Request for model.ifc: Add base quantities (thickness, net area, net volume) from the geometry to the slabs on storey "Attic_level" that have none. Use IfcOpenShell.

First a look at what the model holds.

```python
import ifcopenshell
import ifcopenshell.util.element
import ifcopenshell.util.unit

model = ifcopenshell.open("model.ifc")
print(model.schema)
for unit_type in ("LENGTHUNIT", "AREAUNIT", "VOLUMEUNIT"):
    print(unit_type, ifcopenshell.util.unit.calculate_unit_scale(model, unit_type))
storey = next(s for s in model.by_type("IfcBuildingStorey") if s.Name == "Attic_level")
slabs = [e for e in ifcopenshell.util.element.get_decomposition(storey) if e.is_a("IfcSlab")]
for e in sorted(slabs, key=lambda e: e.id()):
    print(e.id(), e.is_a(), e.Name, list(ifcopenshell.util.element.get_psets(e, qtos_only=True)), sep=" | ")
```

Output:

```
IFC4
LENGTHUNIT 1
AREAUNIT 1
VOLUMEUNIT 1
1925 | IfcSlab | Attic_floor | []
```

```python
import ifcopenshell
import ifcopenshell.api.pset
import ifcopenshell.geom
import ifcopenshell.util.element
import ifcopenshell.util.shape
import ifcopenshell.util.unit

model = ifcopenshell.open("model.ifc")
unit_scale = ifcopenshell.util.unit.calculate_unit_scale(model)
area_scale = ifcopenshell.util.unit.calculate_unit_scale(model, "AREAUNIT")
volume_scale = ifcopenshell.util.unit.calculate_unit_scale(model, "VOLUMEUNIT")
settings = ifcopenshell.geom.settings()

storey = next(s for s in model.by_type("IfcBuildingStorey") if s.Name == "Attic_level")
slabs = [e for e in ifcopenshell.util.element.get_decomposition(storey) if e.is_a("IfcSlab")]

for e in sorted(slabs, key=lambda e: e.id()):
    if ifcopenshell.util.element.get_psets(e, qtos_only=True, should_inherit=False):
        continue
    # Geometry comes back in metres, in the element's own axes.
    shape = ifcopenshell.geom.create_shape(settings, e)
    values = {
        "Width": ifcopenshell.util.shape.get_z(shape.geometry) / unit_scale,
        "NetArea": ifcopenshell.util.shape.get_footprint_area(shape.geometry) / area_scale,
        "NetVolume": ifcopenshell.util.shape.get_volume(shape.geometry) / volume_scale,
    }
    qto = ifcopenshell.api.pset.add_qto(model, product=e, name="Qto_SlabBaseQuantities")
    ifcopenshell.api.pset.edit_qto(model, qto=qto, properties=values)
    print(e.id(), {k: round(v, 3) for k, v in values.items()})

model.write("model_rev.ifc")
```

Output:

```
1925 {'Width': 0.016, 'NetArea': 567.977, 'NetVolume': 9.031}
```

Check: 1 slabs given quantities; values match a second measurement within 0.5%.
